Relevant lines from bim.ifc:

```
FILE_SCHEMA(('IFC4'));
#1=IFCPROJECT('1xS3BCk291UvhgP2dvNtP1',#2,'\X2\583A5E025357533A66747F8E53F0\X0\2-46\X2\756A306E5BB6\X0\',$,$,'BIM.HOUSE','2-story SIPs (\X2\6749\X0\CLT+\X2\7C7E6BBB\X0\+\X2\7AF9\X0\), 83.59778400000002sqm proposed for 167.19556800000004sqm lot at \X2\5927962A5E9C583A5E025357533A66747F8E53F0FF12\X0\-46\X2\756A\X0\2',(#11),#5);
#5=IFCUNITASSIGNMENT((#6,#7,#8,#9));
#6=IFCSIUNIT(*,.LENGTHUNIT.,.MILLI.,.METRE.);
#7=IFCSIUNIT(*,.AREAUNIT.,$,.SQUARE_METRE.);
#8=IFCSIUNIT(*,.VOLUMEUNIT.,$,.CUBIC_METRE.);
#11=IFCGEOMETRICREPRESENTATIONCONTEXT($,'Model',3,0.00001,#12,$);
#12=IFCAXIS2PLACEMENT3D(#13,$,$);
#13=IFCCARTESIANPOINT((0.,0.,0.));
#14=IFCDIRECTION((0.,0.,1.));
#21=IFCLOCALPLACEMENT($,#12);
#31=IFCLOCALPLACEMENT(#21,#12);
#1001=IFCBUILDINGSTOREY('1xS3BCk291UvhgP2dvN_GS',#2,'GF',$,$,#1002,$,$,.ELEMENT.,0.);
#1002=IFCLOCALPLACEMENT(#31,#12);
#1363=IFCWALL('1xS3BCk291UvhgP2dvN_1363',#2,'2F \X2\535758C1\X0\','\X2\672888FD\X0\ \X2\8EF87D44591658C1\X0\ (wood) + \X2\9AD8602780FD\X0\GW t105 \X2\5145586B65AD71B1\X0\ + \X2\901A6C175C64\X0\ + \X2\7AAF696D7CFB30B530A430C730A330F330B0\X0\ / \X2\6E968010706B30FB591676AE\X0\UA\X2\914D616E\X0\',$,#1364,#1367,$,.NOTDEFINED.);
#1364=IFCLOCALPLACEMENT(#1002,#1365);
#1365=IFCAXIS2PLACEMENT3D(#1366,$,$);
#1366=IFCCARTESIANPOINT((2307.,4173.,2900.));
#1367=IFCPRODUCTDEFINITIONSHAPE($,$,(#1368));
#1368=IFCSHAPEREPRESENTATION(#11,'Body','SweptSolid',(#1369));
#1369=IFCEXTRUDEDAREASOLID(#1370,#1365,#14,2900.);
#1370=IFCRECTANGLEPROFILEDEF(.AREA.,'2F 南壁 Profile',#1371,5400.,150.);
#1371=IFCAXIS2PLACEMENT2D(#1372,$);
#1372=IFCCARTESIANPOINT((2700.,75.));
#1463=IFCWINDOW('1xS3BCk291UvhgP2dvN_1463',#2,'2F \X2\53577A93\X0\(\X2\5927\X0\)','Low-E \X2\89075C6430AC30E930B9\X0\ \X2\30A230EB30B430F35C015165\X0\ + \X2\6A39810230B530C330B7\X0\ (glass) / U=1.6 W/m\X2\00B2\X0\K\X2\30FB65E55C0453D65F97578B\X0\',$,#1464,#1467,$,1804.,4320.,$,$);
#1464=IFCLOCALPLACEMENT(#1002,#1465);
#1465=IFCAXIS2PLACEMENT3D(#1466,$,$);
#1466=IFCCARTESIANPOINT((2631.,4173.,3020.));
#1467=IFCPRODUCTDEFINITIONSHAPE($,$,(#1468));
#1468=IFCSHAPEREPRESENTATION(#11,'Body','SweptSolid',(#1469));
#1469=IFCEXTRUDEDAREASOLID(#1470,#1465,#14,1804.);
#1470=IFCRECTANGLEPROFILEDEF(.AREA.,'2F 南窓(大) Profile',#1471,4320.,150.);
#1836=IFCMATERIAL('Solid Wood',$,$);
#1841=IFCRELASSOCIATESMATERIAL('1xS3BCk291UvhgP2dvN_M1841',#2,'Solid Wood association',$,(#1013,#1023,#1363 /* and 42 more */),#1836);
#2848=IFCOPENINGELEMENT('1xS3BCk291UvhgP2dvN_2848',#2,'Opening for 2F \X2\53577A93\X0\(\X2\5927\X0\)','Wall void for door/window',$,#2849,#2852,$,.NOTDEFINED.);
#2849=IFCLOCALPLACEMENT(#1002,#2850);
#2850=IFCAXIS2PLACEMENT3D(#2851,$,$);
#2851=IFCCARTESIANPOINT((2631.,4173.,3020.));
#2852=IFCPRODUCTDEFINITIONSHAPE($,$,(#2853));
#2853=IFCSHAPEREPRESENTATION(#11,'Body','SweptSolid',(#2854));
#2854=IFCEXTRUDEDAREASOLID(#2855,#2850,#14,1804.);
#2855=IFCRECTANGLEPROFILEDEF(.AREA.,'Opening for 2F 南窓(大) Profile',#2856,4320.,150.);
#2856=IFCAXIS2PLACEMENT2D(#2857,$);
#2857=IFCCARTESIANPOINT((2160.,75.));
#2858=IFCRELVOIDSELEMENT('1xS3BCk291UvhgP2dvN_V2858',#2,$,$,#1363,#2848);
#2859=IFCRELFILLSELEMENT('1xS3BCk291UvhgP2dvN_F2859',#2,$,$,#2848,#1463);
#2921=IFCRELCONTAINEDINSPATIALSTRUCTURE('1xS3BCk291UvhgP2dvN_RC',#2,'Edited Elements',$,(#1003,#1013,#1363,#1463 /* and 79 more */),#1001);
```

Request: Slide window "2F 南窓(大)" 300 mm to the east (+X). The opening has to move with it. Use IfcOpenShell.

```python
import ifcopenshell
import ifcopenshell.api.geometry
import ifcopenshell.util.placement
import ifcopenshell.util.unit

model = ifcopenshell.open("bim.ifc")
unit_scale = ifcopenshell.util.unit.calculate_unit_scale(model)

window = model.by_guid("1xS3BCk291UvhgP2dvN_1463")
opening = window.FillsVoids[0].RelatingOpeningElement
wall = opening.VoidsElements[0].RelatingBuildingElement

wall_matrix = ifcopenshell.util.placement.get_local_placement(wall.ObjectPlacement)
shift = wall_matrix[:3, 0] * 0.3 / unit_scale
before = ifcopenshell.util.placement.get_local_placement(window.ObjectPlacement)[:3, 3].copy()

# The window is not placed relative to its opening, so move both.
for product in (opening, window):
    matrix = ifcopenshell.util.placement.get_local_placement(product.ObjectPlacement)
    matrix[:3, 3] += shift
    ifcopenshell.api.geometry.edit_object_placement(model, product=product, matrix=matrix, is_si=False)

after = ifcopenshell.util.placement.get_local_placement(window.ObjectPlacement)[:3, 3]
print("window moved by", (after - before).round(3) + 0.0)

model.write("bim_updated.ifc")
```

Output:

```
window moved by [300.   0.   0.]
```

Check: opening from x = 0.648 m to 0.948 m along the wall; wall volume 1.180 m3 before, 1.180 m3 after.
